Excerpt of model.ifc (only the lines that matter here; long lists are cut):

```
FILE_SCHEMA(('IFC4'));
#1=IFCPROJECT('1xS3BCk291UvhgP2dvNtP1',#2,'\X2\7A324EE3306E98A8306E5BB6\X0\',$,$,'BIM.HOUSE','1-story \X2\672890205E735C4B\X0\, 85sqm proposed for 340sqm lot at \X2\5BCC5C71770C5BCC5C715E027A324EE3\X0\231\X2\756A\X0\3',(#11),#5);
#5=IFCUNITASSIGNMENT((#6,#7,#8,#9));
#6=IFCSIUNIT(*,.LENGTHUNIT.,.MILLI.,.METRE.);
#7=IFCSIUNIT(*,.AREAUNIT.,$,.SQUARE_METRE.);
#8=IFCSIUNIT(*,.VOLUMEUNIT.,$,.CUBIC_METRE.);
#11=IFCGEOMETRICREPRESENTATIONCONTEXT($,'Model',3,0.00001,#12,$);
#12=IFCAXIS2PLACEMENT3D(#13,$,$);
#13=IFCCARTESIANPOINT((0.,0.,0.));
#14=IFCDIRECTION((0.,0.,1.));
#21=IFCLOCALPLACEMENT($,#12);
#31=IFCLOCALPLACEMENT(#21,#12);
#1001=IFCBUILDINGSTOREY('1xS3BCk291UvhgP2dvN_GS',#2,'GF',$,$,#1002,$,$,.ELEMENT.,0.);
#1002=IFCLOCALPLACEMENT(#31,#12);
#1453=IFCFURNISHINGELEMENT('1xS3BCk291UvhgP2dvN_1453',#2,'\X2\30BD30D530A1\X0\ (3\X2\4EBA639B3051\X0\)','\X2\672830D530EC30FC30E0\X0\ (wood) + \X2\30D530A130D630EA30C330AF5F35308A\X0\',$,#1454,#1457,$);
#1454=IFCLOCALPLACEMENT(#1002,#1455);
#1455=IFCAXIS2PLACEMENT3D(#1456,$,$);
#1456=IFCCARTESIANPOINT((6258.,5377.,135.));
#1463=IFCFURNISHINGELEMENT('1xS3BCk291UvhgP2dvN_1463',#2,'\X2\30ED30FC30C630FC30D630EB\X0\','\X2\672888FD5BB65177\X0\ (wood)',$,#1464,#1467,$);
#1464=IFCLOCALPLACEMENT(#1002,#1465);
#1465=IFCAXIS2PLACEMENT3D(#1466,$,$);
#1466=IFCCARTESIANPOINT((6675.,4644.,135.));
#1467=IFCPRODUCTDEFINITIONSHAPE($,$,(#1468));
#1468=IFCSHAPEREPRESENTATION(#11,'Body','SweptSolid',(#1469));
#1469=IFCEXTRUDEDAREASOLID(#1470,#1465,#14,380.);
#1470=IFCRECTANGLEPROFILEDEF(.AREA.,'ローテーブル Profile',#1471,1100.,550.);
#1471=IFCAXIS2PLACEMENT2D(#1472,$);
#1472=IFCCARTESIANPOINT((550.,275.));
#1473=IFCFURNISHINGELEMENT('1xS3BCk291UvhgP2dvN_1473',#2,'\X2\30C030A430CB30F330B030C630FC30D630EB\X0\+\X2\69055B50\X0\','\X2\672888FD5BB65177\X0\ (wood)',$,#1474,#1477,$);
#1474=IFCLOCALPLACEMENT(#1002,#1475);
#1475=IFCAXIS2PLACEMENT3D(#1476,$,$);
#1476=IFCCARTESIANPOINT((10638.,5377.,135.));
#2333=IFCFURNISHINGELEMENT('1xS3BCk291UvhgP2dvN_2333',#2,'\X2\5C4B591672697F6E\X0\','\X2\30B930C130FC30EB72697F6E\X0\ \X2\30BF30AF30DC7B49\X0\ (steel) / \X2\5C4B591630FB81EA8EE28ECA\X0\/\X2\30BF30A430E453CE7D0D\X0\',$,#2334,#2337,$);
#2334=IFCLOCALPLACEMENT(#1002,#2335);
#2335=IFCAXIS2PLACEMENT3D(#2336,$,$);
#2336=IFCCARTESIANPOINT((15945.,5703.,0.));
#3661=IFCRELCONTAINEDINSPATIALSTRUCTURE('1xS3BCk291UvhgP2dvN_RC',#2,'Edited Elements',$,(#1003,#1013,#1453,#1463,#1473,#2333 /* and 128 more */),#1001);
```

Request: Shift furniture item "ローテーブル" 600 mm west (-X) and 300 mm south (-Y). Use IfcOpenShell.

```python
import ifcopenshell
import ifcopenshell.api.geometry
import ifcopenshell.util.placement
import ifcopenshell.util.unit

model = ifcopenshell.open("model.ifc")
unit_scale = ifcopenshell.util.unit.calculate_unit_scale(model)

item = model.by_guid("1xS3BCk291UvhgP2dvN_1463")
matrix = ifcopenshell.util.placement.get_local_placement(item.ObjectPlacement)
matrix[0, 3] -= 0.6 / unit_scale
matrix[1, 3] -= 0.3 / unit_scale
ifcopenshell.api.geometry.edit_object_placement(model, product=item, matrix=matrix, is_si=False)

print(ifcopenshell.util.placement.get_local_placement(item.ObjectPlacement).round(3) + 0.0)

model.write("model-out.ifc")
```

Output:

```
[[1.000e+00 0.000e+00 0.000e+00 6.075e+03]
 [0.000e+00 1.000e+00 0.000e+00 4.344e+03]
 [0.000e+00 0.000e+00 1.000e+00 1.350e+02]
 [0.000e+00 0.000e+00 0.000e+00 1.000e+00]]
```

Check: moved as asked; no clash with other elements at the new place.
